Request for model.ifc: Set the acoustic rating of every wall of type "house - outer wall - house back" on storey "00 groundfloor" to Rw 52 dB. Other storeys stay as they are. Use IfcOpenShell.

First a look at what the model holds.

```python
import ifcopenshell
import ifcopenshell.util.element

model = ifcopenshell.open("model.ifc")
print(model.schema)
storey = next(s for s in model.by_type("IfcBuildingStorey") if s.Name == "00 groundfloor")
walls = [e for e in ifcopenshell.util.element.get_decomposition(storey) if e.is_a("IfcWall")]
seen = {}
for e in walls:
    element_type = ifcopenshell.util.element.get_type(e)
    key = (element_type.Name if element_type != e and element_type else None, ifcopenshell.util.element.get_pset(e, "Pset_WallCommon", "AcousticRating"))
    seen[key] = seen.get(key, 0) + 1
for (name, value), count in sorted(seen.items(), key=str):
    print(count, "x", name, "|", value)
```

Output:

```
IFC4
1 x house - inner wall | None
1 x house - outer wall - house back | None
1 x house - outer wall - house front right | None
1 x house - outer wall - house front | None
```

```python
import ifcopenshell
import ifcopenshell.api.pset
import ifcopenshell.util.element

model = ifcopenshell.open("model.ifc")

storey = next(s for s in model.by_type("IfcBuildingStorey") if s.Name == "00 groundfloor")
walls = [e for e in ifcopenshell.util.element.get_decomposition(storey) if e.is_a("IfcWall")]

count = 0
for e in walls:
    element_type = ifcopenshell.util.element.get_type(e)
    if element_type in (None, e) or element_type.Name != "house - outer wall - house back":
        continue
    # add_pset returns the element's existing set when there is one.
    pset = ifcopenshell.api.pset.add_pset(model, product=e, name="Pset_WallCommon")
    ifcopenshell.api.pset.edit_pset(model, pset=pset, properties={"AcousticRating": "Rw 52 dB"})
    count += 1

print(count, "walls updated")

model.write("model_v2.ifc")
```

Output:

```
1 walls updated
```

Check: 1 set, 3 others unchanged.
